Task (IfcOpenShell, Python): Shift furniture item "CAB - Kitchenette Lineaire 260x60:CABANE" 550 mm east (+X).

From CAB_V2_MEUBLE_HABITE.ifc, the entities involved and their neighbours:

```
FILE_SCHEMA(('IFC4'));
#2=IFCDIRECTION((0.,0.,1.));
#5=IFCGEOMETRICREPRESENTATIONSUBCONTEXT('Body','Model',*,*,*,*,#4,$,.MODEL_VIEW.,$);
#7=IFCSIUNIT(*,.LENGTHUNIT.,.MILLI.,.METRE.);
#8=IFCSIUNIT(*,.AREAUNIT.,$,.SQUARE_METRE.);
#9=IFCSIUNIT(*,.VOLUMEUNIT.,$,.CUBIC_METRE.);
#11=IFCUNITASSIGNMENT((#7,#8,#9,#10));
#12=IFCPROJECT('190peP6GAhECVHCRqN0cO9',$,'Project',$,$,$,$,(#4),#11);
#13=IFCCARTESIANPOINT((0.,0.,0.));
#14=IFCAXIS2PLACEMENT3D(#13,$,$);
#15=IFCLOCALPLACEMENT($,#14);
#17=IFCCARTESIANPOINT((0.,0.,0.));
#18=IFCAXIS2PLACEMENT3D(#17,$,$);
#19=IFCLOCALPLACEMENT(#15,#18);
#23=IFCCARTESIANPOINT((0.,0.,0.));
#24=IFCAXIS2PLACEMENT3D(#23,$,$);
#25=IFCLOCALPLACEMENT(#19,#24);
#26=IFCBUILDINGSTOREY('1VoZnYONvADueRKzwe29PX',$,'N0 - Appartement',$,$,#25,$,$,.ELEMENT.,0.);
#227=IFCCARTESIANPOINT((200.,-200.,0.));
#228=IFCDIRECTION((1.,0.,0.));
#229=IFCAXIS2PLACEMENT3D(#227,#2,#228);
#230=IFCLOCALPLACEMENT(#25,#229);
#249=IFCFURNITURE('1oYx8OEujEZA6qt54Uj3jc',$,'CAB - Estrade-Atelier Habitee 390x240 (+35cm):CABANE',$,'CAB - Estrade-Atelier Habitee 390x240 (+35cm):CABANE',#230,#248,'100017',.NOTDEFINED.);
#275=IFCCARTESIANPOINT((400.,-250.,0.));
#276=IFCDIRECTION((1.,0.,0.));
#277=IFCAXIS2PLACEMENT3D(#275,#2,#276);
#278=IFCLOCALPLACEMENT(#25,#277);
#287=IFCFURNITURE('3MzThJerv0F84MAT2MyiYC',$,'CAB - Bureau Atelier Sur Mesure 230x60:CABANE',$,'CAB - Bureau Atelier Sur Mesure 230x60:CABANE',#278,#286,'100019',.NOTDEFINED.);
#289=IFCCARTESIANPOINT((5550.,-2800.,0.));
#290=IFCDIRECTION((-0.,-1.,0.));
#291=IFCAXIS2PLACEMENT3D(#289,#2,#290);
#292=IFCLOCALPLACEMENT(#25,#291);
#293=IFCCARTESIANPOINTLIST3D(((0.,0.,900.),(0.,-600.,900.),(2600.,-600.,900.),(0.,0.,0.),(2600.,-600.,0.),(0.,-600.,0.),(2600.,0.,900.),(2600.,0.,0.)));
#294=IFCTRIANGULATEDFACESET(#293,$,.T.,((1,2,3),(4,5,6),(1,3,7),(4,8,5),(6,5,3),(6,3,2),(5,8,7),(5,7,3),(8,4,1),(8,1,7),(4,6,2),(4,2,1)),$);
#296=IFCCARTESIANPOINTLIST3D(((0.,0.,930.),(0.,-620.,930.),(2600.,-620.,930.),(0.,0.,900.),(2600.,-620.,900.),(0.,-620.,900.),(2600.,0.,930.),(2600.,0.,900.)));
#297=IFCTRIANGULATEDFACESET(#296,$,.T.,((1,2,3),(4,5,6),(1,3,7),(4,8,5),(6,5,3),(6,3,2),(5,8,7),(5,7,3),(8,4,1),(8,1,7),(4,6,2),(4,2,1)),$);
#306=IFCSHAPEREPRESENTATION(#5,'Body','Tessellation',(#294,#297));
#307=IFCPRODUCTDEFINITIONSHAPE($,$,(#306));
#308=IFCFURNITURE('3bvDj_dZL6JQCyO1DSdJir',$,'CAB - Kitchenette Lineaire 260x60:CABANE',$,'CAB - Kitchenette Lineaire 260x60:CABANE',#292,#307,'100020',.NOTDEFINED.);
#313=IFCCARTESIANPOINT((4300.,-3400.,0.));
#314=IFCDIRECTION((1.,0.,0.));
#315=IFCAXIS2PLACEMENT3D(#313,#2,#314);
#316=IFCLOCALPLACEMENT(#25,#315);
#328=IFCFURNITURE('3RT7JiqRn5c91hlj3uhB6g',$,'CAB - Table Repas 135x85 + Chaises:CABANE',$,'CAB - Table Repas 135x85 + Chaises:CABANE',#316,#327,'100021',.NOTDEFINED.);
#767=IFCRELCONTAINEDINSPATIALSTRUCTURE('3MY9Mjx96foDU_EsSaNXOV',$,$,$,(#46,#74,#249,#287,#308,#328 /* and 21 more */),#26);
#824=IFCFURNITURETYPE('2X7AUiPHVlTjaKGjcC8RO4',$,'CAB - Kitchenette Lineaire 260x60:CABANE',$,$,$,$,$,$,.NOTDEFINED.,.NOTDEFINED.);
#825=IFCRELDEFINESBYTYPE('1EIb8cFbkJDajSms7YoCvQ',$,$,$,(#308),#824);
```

```python
import ifcopenshell
import ifcopenshell.api.geometry
import ifcopenshell.util.placement
import ifcopenshell.util.unit

model = ifcopenshell.open("CAB_V2_MEUBLE_HABITE.ifc")
unit_scale = ifcopenshell.util.unit.calculate_unit_scale(model)

item = model.by_id(308)
matrix = ifcopenshell.util.placement.get_local_placement(item.ObjectPlacement)
matrix[0, 3] += 0.55 / unit_scale
ifcopenshell.api.geometry.edit_object_placement(model, product=item, matrix=matrix, is_si=False)

print(ifcopenshell.util.placement.get_local_placement(item.ObjectPlacement).round(3) + 0.0)

model.write("CAB_V2_MEUBLE_HABITE_edited.ifc")
```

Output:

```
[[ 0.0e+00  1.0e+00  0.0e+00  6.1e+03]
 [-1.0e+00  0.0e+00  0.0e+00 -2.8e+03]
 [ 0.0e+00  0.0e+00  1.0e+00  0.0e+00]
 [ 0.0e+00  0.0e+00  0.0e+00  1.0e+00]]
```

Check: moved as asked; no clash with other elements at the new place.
